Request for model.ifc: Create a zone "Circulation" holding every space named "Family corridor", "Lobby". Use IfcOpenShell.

First a look at what the model holds.

```python
import ifcopenshell

model = ifcopenshell.open("model.ifc")
print(model.schema)
seen = {}
for space in model.by_type("IfcSpace"):
    seen[space.LongName] = seen.get(space.LongName, 0) + 1
for name, count in sorted(seen.items(), key=str):
    print(count, "x", name)
print("zones:", [z.Name for z in model.by_type("IfcZone")][:20])
```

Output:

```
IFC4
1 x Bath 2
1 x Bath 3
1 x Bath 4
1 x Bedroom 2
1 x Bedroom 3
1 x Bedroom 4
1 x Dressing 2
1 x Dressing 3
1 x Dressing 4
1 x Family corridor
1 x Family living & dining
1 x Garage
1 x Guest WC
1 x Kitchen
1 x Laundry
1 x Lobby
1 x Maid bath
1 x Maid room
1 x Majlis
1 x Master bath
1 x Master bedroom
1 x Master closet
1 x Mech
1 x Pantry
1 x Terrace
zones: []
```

```python
import ifcopenshell
import ifcopenshell.api.group
import ifcopenshell.api.root

model = ifcopenshell.open("model.ifc")

names = {"Family corridor", "Lobby"}
spaces = [s for s in model.by_type("IfcSpace") if s.LongName in names]

zone = ifcopenshell.api.root.create_entity(model, ifc_class="IfcZone", name="Circulation")
ifcopenshell.api.group.assign_group(model, products=spaces, group=zone)
print(len(spaces), "spaces in", zone.Name)

model.write("model-out.ifc")
```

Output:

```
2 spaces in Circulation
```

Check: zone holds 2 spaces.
